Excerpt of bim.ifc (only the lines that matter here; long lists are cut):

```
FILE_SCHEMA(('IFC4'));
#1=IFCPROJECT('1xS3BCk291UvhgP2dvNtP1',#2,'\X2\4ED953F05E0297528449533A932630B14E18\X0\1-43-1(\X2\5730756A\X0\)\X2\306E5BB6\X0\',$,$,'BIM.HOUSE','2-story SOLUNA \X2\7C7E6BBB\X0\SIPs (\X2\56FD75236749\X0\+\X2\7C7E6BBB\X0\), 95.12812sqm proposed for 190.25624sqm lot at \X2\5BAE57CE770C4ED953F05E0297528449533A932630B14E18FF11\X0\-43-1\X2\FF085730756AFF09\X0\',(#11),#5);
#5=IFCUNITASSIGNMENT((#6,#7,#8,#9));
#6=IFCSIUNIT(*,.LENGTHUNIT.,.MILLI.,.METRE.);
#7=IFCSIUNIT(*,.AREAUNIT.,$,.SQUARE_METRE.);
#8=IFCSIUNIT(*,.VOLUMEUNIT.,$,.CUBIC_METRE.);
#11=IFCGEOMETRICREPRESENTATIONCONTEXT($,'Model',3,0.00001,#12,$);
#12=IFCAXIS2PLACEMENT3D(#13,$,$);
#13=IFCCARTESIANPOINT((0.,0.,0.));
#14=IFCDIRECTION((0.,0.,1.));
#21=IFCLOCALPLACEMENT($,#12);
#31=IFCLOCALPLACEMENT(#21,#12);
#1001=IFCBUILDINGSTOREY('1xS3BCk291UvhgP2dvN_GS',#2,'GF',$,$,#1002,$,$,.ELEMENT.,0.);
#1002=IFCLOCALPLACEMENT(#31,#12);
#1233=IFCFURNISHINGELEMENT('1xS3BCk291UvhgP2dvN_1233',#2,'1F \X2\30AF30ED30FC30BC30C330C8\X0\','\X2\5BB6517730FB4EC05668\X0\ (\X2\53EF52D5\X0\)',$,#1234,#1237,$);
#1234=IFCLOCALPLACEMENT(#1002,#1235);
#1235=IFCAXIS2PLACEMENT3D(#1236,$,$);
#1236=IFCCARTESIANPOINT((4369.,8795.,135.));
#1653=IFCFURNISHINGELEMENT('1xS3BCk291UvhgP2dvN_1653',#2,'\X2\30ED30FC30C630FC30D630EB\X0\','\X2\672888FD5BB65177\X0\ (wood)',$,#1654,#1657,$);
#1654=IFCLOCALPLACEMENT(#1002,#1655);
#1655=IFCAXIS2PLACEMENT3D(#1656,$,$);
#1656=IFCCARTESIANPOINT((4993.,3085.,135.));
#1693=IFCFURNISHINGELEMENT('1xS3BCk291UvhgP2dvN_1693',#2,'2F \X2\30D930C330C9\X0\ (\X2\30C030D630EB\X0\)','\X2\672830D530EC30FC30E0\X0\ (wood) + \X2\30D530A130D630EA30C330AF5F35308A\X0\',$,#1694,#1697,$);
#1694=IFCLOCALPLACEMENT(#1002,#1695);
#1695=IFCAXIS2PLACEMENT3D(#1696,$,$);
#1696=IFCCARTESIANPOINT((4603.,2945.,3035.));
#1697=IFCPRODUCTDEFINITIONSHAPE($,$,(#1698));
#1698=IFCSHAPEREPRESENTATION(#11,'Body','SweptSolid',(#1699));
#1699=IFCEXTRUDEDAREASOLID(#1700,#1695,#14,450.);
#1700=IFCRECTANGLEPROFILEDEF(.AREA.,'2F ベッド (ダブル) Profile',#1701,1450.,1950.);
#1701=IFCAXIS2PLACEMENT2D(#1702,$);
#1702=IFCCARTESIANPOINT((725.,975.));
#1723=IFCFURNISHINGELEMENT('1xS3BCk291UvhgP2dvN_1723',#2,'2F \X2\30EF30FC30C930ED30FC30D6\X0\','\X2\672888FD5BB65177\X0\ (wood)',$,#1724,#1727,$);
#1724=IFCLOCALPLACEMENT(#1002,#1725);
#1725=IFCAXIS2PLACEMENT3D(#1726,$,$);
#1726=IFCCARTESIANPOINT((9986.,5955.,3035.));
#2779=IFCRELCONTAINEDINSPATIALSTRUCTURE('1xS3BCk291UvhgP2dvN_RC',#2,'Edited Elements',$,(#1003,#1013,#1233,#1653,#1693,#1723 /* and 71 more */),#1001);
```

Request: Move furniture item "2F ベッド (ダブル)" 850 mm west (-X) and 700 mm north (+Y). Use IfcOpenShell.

```python
import ifcopenshell
import ifcopenshell.api.geometry
import ifcopenshell.util.placement
import ifcopenshell.util.unit

model = ifcopenshell.open("bim.ifc")
unit_scale = ifcopenshell.util.unit.calculate_unit_scale(model)

item = model.by_guid("1xS3BCk291UvhgP2dvN_1693")
matrix = ifcopenshell.util.placement.get_local_placement(item.ObjectPlacement)
matrix[0, 3] -= 0.85 / unit_scale
matrix[1, 3] += 0.7 / unit_scale
ifcopenshell.api.geometry.edit_object_placement(model, product=item, matrix=matrix, is_si=False)

print(ifcopenshell.util.placement.get_local_placement(item.ObjectPlacement).round(3) + 0.0)

model.write("bim_updated.ifc")
```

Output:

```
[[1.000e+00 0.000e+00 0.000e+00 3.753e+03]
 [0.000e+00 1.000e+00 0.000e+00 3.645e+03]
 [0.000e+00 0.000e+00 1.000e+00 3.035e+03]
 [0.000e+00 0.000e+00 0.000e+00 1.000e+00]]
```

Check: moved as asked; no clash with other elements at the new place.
